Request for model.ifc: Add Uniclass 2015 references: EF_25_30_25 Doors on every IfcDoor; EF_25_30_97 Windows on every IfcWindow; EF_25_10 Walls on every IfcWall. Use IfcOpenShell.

First a look at what the model holds.

```python
import ifcopenshell

model = ifcopenshell.open("model.ifc")
print(model.schema)
print("classifications:", [c.Name for c in model.by_type("IfcClassification")])
for ifc_class in ("IfcDoor", "IfcRoof", "IfcStair", "IfcWall", "IfcWindow"):
    print(ifc_class, len(model.by_type(ifc_class)))
```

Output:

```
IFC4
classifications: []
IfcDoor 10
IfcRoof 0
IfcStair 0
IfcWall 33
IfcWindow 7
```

```python
import ifcopenshell
import ifcopenshell.api.classification

model = ifcopenshell.open("model.ifc")

system = ifcopenshell.api.classification.add_classification(model, classification="Uniclass 2015")

codes = {
    "IfcDoor": ("EF_25_30_25", "Doors"),
    "IfcWindow": ("EF_25_30_97", "Windows"),
    "IfcWall": ("EF_25_10", "Walls"),
}
for ifc_class, (code, name) in codes.items():
    products = model.by_type(ifc_class)
    ifcopenshell.api.classification.add_reference(
        model, products=products, classification=system, identification=code, name=name
    )
    print(code, len(products))

model.write("model-out.ifc")
```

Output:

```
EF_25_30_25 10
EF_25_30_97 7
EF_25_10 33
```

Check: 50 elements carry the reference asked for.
